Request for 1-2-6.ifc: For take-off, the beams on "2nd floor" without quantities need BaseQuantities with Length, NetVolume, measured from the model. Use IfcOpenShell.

First a look at what the model holds.

```python
import ifcopenshell
import ifcopenshell.util.element
import ifcopenshell.util.unit

model = ifcopenshell.open("1-2-6.ifc")
print(model.schema)
for unit_type in ("LENGTHUNIT", "AREAUNIT", "VOLUMEUNIT"):
    print(unit_type, ifcopenshell.util.unit.calculate_unit_scale(model, unit_type))
storey = next(s for s in model.by_type("IfcBuildingStorey") if s.Name == "2nd floor")
beams = [e for e in ifcopenshell.util.element.get_decomposition(storey) if e.is_a("IfcBeam")]
for e in sorted(beams, key=lambda e: e.id()):
    print(e.id(), e.is_a(), e.Name, list(ifcopenshell.util.element.get_psets(e, qtos_only=True)), sep=" | ")
```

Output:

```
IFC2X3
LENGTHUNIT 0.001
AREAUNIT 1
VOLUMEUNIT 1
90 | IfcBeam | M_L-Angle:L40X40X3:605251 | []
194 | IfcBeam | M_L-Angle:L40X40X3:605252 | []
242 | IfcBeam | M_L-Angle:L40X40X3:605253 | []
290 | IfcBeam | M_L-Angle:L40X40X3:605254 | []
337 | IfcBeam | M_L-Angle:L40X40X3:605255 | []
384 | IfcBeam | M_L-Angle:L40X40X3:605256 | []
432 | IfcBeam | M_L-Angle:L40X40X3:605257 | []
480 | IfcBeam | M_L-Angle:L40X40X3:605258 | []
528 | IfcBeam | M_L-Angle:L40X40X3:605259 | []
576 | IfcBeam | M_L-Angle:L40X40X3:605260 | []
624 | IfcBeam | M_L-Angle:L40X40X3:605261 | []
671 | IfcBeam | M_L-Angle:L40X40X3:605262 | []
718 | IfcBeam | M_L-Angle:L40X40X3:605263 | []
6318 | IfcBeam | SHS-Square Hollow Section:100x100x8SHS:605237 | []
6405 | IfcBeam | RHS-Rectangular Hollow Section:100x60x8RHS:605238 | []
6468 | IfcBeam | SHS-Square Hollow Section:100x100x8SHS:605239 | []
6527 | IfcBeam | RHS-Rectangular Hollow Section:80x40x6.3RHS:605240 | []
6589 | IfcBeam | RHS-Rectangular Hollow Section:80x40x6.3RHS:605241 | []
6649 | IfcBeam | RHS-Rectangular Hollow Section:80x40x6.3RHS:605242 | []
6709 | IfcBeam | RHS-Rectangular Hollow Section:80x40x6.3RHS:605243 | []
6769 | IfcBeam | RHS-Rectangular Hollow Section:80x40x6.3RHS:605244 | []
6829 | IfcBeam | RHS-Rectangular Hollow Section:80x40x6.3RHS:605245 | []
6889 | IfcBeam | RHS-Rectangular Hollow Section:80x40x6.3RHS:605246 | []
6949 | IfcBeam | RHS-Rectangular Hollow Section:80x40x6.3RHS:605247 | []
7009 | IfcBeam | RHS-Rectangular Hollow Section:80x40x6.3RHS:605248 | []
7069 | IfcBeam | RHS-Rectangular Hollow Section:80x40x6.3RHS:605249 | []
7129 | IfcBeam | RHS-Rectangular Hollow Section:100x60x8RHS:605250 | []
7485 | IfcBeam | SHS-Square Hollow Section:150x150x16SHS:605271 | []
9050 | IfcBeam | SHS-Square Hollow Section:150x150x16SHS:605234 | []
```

```python
import ifcopenshell
import ifcopenshell.api.pset
import ifcopenshell.geom
import ifcopenshell.util.element
import ifcopenshell.util.shape
import ifcopenshell.util.unit

model = ifcopenshell.open("1-2-6.ifc")
unit_scale = ifcopenshell.util.unit.calculate_unit_scale(model)
volume_scale = ifcopenshell.util.unit.calculate_unit_scale(model, "VOLUMEUNIT")
settings = ifcopenshell.geom.settings()

storey = next(s for s in model.by_type("IfcBuildingStorey") if s.Name == "2nd floor")
beams = [e for e in ifcopenshell.util.element.get_decomposition(storey) if e.is_a("IfcBeam")]

for e in sorted(beams, key=lambda e: e.id()):
    if ifcopenshell.util.element.get_psets(e, qtos_only=True, should_inherit=False):
        continue
    # Geometry comes back in metres, in the element's own axes.
    shape = ifcopenshell.geom.create_shape(settings, e)
    values = {
        "Length": ifcopenshell.util.shape.get_max_xyz(shape.geometry) / unit_scale,
        "NetVolume": ifcopenshell.util.shape.get_volume(shape.geometry) / volume_scale,
    }
    qto = ifcopenshell.api.pset.add_qto(model, product=e, name="BaseQuantities")
    ifcopenshell.api.pset.edit_qto(model, qto=qto, properties=values)
    print(e.id(), {k: round(v, 3) for k, v in values.items()})

model.write("1-2-6_edited.ifc")
```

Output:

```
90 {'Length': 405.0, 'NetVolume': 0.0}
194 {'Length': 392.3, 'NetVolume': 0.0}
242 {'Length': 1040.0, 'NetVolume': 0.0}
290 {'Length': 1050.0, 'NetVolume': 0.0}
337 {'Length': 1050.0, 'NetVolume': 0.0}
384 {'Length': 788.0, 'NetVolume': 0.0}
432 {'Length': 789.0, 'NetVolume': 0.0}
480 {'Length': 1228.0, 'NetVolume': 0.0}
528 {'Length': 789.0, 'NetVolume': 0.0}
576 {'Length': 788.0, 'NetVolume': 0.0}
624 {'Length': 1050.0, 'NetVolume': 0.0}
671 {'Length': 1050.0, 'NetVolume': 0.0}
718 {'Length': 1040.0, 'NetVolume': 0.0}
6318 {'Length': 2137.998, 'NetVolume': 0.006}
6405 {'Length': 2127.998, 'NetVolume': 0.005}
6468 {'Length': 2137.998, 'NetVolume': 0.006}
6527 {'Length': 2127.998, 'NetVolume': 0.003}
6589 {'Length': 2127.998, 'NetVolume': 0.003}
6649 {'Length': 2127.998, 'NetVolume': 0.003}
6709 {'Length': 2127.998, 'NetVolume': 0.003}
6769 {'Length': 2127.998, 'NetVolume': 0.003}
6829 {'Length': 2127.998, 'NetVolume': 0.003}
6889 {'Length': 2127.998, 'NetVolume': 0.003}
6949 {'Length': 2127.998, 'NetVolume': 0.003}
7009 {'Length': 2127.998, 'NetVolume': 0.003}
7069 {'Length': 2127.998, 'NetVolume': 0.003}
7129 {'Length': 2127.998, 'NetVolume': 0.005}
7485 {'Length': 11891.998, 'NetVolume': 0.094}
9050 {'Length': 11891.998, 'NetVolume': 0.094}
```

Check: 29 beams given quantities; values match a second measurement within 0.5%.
